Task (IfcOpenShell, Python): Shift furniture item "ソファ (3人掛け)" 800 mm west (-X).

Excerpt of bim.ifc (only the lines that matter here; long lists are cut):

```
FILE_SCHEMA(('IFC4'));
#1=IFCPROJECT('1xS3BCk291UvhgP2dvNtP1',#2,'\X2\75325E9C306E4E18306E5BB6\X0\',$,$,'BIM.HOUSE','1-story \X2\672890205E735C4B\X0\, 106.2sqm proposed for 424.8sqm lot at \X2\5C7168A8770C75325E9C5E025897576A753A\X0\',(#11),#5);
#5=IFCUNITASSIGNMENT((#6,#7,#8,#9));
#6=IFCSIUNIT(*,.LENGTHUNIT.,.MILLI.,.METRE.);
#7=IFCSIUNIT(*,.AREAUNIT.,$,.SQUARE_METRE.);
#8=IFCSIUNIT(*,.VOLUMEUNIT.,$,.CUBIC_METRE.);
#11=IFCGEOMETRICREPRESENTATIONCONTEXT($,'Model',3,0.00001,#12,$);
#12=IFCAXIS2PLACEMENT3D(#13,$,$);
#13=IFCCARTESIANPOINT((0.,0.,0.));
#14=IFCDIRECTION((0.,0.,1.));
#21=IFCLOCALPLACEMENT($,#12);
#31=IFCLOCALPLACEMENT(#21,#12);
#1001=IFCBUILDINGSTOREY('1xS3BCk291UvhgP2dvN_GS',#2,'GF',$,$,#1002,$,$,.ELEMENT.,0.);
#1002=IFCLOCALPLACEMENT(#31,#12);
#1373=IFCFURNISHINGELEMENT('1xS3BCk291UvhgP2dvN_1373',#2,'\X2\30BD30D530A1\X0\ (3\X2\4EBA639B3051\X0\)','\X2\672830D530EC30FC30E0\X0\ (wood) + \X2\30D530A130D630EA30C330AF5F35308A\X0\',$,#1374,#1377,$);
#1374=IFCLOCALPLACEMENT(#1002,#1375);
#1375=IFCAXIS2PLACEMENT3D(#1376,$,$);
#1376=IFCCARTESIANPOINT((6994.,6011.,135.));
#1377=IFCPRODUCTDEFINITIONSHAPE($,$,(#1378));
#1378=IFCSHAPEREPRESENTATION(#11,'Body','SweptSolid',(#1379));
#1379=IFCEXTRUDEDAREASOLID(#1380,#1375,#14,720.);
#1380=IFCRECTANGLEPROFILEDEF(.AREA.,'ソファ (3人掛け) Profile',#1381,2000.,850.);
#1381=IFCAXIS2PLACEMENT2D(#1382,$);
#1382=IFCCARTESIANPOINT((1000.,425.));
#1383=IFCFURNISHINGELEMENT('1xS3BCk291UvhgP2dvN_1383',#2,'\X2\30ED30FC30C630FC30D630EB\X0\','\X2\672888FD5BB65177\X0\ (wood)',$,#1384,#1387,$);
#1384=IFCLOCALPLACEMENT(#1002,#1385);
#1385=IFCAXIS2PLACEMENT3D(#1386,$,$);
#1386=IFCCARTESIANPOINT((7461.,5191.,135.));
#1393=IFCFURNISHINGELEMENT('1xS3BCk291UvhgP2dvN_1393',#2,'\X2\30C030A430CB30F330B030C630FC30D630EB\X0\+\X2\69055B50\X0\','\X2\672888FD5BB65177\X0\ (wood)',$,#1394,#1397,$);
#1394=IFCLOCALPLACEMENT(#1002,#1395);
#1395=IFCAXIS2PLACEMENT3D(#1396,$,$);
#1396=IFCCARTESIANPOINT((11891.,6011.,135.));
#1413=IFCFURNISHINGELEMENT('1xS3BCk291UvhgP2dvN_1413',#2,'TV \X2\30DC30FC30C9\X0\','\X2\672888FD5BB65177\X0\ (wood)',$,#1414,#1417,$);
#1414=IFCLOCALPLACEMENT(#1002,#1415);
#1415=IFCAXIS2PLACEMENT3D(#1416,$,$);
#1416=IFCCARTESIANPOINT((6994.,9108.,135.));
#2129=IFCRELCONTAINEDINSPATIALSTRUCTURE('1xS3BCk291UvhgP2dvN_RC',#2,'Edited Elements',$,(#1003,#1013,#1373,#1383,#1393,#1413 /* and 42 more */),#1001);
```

```python
import ifcopenshell
import ifcopenshell.api.geometry
import ifcopenshell.util.placement
import ifcopenshell.util.unit

model = ifcopenshell.open("bim.ifc")
unit_scale = ifcopenshell.util.unit.calculate_unit_scale(model)

item = model.by_guid("1xS3BCk291UvhgP2dvN_1373")
matrix = ifcopenshell.util.placement.get_local_placement(item.ObjectPlacement)
matrix[0, 3] -= 0.8 / unit_scale
ifcopenshell.api.geometry.edit_object_placement(model, product=item, matrix=matrix, is_si=False)

print(ifcopenshell.util.placement.get_local_placement(item.ObjectPlacement).round(3) + 0.0)

model.write("bim_rev.ifc")
```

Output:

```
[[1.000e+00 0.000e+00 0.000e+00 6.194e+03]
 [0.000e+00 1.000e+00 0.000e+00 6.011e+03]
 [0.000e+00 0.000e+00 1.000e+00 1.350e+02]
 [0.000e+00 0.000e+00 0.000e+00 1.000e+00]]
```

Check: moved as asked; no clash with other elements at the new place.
